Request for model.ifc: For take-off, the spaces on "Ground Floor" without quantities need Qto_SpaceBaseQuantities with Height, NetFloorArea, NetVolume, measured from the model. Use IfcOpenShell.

First a look at what the model holds.

```python
import ifcopenshell
import ifcopenshell.util.element
import ifcopenshell.util.unit

model = ifcopenshell.open("model.ifc")
print(model.schema)
for unit_type in ("LENGTHUNIT", "AREAUNIT", "VOLUMEUNIT"):
    print(unit_type, ifcopenshell.util.unit.calculate_unit_scale(model, unit_type))
storey = next(s for s in model.by_type("IfcBuildingStorey") if s.Name == "Ground Floor")
spaces = [e for e in ifcopenshell.util.element.get_decomposition(storey) if e.is_a("IfcSpace")]
for e in sorted(spaces, key=lambda e: e.id()):
    print(e.id(), e.is_a(), e.Name, list(ifcopenshell.util.element.get_psets(e, qtos_only=True)), sep=" | ")
```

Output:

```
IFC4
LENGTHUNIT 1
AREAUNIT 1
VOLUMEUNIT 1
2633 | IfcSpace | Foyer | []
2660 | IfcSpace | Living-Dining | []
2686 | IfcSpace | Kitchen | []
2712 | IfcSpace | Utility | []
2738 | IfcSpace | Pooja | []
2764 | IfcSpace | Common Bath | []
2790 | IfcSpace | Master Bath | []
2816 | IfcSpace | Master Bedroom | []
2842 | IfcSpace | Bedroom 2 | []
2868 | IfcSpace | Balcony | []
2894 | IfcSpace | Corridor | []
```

```python
import ifcopenshell
import ifcopenshell.api.pset
import ifcopenshell.geom
import ifcopenshell.util.element
import ifcopenshell.util.shape
import ifcopenshell.util.unit

model = ifcopenshell.open("model.ifc")
unit_scale = ifcopenshell.util.unit.calculate_unit_scale(model)
area_scale = ifcopenshell.util.unit.calculate_unit_scale(model, "AREAUNIT")
volume_scale = ifcopenshell.util.unit.calculate_unit_scale(model, "VOLUMEUNIT")
settings = ifcopenshell.geom.settings()

storey = next(s for s in model.by_type("IfcBuildingStorey") if s.Name == "Ground Floor")
spaces = [e for e in ifcopenshell.util.element.get_decomposition(storey) if e.is_a("IfcSpace")]

for e in sorted(spaces, key=lambda e: e.id()):
    if ifcopenshell.util.element.get_psets(e, qtos_only=True, should_inherit=False):
        continue
    # Geometry comes back in metres, in the element's own axes.
    shape = ifcopenshell.geom.create_shape(settings, e)
    values = {
        "Height": ifcopenshell.util.shape.get_z(shape.geometry) / unit_scale,
        "NetFloorArea": ifcopenshell.util.shape.get_footprint_area(shape.geometry) / area_scale,
        "NetVolume": ifcopenshell.util.shape.get_volume(shape.geometry) / volume_scale,
    }
    qto = ifcopenshell.api.pset.add_qto(model, product=e, name="Qto_SpaceBaseQuantities")
    ifcopenshell.api.pset.edit_qto(model, qto=qto, properties=values)
    print(e.id(), {k: round(v, 3) for k, v in values.items()})

model.write("model-out.ifc")
```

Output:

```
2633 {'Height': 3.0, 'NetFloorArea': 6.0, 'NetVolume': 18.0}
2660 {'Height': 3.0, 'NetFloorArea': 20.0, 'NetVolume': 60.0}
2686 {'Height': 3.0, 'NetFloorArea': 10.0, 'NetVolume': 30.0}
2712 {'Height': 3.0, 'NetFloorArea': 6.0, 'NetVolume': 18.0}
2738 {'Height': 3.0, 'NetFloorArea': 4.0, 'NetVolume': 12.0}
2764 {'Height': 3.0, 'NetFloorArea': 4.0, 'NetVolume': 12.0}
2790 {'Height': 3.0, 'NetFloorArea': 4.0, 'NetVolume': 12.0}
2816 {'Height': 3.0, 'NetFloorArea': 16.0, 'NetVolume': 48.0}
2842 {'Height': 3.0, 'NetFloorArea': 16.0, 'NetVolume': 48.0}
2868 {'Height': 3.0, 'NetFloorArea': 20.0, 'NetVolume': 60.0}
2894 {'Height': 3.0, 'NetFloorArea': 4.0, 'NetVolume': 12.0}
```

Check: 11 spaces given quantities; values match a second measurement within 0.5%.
